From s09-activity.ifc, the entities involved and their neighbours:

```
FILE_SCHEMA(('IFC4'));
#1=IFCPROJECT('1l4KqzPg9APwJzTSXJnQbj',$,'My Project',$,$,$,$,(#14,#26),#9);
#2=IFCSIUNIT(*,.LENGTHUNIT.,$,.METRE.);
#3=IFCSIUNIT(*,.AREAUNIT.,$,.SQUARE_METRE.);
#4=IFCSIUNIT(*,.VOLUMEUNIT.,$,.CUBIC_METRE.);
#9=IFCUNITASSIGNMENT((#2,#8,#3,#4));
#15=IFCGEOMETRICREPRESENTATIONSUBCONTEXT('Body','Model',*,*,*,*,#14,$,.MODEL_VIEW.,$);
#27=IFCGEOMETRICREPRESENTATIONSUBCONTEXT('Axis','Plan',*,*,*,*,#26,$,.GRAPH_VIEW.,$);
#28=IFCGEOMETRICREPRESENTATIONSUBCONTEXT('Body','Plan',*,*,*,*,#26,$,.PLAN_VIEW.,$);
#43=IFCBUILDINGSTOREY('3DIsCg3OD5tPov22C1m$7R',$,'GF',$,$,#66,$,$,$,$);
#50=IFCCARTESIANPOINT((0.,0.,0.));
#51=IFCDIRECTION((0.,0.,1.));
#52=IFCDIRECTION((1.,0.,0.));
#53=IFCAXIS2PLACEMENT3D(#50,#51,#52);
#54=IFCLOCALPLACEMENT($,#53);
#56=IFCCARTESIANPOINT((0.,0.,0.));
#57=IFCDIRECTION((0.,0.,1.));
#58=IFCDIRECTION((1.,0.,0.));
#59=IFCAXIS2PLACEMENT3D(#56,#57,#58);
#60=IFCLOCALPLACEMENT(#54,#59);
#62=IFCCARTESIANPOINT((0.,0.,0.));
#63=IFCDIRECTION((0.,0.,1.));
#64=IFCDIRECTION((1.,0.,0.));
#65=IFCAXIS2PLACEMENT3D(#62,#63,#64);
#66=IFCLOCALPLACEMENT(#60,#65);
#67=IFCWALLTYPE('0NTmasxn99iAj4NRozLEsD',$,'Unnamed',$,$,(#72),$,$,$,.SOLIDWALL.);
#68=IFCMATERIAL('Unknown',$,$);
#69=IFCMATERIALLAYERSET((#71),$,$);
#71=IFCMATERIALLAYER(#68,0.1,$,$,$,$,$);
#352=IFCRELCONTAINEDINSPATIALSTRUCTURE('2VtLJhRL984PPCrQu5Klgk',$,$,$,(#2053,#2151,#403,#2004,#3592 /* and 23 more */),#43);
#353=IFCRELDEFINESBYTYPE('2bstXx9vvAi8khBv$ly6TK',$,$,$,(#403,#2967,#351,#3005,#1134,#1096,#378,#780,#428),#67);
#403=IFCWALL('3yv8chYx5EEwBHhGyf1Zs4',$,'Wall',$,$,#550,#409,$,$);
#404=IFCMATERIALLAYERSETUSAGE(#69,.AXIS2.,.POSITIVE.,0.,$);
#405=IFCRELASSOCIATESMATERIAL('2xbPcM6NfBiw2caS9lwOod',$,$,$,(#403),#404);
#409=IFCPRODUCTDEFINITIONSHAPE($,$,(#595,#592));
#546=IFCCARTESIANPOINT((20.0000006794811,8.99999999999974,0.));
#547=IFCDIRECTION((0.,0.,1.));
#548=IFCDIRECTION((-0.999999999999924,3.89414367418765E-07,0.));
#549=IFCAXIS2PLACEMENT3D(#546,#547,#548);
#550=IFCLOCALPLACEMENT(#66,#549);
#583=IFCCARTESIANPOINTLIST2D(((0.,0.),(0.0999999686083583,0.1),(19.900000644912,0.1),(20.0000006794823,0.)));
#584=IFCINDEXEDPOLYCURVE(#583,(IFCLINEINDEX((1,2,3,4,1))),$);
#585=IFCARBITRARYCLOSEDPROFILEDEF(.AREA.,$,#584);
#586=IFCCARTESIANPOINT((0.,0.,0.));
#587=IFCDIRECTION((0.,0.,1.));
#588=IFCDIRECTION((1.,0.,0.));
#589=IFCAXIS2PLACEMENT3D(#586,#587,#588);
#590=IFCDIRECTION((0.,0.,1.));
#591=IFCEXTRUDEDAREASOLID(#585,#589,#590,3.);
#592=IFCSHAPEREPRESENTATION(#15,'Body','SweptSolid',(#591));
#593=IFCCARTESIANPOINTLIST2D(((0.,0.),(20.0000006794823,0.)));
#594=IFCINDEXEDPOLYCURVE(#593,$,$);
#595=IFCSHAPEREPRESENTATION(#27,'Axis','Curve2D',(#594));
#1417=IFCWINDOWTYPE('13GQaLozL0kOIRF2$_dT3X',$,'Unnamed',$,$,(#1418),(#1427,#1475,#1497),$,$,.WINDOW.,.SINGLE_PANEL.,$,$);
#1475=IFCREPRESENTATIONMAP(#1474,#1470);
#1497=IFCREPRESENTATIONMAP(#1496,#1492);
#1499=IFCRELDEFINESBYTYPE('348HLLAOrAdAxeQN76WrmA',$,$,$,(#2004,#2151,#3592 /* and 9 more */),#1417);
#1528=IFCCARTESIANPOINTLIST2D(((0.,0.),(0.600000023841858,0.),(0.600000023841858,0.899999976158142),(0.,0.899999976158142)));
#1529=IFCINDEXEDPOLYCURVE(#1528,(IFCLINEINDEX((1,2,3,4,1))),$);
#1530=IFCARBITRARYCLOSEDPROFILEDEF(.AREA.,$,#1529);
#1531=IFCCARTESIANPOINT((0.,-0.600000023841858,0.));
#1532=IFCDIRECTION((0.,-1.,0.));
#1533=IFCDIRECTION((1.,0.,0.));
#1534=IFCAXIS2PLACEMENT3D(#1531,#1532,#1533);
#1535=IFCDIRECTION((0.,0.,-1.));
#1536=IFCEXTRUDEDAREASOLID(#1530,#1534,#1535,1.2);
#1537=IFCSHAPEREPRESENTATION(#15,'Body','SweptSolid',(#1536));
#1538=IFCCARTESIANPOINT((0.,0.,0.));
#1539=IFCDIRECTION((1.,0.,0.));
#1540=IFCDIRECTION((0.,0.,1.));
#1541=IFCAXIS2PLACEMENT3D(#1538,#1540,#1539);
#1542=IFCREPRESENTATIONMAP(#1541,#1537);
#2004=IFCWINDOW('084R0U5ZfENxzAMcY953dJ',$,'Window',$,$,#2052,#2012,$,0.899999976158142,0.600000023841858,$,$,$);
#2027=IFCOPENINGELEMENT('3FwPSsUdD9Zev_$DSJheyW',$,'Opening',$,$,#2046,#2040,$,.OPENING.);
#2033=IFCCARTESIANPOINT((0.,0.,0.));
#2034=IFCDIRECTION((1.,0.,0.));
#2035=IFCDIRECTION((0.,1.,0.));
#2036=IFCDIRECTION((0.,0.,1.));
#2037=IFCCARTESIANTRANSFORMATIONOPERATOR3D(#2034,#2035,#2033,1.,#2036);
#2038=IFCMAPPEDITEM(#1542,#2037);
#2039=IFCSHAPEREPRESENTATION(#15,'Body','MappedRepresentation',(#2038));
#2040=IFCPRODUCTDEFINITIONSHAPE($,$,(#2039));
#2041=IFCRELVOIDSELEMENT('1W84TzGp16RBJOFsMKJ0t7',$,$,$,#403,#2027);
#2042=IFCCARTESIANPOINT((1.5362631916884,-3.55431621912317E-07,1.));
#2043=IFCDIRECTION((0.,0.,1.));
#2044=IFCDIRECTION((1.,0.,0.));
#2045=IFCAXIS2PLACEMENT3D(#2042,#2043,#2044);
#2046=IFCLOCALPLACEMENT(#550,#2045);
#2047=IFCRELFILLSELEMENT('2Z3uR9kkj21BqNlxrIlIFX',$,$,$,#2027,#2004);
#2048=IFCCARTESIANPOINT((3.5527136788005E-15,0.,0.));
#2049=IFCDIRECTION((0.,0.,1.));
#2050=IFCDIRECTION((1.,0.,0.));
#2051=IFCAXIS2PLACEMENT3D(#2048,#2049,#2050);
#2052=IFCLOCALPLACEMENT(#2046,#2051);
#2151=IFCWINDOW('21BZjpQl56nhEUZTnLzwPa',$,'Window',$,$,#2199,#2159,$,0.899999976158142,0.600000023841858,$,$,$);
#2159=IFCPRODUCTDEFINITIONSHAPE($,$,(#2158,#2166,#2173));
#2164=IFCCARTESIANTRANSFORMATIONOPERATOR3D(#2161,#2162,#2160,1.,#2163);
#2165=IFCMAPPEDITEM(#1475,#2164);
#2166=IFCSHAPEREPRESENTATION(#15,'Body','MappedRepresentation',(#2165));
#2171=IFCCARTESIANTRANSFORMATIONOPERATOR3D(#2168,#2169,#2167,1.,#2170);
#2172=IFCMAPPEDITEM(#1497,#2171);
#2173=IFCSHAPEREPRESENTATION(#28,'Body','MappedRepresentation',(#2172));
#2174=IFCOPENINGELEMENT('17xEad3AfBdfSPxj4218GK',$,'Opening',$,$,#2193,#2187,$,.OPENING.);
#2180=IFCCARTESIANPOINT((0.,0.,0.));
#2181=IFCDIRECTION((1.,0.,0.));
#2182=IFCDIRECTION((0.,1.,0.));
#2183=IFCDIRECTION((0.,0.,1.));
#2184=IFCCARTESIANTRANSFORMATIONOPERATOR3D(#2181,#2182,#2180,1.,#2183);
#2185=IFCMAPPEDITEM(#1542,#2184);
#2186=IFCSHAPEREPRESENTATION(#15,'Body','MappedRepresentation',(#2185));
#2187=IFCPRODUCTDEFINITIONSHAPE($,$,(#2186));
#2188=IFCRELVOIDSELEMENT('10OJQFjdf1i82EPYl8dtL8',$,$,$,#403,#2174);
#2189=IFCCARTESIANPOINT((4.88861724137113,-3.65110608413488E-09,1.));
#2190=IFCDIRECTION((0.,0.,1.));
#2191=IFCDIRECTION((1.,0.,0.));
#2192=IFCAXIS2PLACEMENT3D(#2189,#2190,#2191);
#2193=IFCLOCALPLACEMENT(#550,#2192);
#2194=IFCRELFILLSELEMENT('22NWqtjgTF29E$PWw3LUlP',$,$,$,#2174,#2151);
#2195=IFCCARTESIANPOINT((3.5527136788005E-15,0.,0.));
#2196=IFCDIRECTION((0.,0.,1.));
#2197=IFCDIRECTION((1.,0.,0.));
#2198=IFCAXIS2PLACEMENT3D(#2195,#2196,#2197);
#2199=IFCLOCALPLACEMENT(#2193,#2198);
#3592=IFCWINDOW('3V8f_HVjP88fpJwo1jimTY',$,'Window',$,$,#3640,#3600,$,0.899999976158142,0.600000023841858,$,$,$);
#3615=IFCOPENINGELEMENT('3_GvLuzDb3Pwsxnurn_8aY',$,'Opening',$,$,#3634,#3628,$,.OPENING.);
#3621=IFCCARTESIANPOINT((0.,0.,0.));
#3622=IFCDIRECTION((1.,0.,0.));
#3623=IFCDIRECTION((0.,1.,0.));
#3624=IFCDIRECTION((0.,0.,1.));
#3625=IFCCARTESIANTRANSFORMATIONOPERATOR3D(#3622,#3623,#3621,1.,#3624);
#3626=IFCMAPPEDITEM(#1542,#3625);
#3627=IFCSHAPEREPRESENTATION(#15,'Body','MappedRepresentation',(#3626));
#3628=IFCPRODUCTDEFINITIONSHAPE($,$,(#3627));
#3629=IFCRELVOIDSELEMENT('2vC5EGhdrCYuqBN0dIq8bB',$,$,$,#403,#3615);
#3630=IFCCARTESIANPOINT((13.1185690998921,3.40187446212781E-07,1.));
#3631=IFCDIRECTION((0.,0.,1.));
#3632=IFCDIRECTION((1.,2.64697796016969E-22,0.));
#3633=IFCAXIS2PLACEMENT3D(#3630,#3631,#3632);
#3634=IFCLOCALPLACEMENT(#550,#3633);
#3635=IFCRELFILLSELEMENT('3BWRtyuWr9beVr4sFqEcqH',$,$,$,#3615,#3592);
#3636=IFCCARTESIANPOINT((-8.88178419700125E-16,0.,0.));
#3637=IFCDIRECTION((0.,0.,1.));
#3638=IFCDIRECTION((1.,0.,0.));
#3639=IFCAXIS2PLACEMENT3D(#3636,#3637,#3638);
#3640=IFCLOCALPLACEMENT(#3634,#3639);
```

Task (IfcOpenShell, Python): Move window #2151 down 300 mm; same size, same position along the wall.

```python
import numpy as np
import ifcopenshell
import ifcopenshell.api.geometry
import ifcopenshell.util.placement
import ifcopenshell.util.unit

model = ifcopenshell.open("s09-activity.ifc")
unit_scale = ifcopenshell.util.unit.calculate_unit_scale(model)

window = model.by_id(2151)
opening = window.FillsVoids[0].RelatingOpeningElement
dz = -0.3

shift = np.array([0.0, 0.0, dz])
# The window is placed relative to its opening, so it follows when the opening moves.
matrix = ifcopenshell.util.placement.get_local_placement(opening.ObjectPlacement)
matrix[:3, 3] += shift
ifcopenshell.api.geometry.edit_object_placement(
    model, product=opening, matrix=matrix, is_si=False, should_transform_children=True
)

print(f"moved by {dz * unit_scale:+.3f} m")

model.write("s09-activity_updated.ifc")
```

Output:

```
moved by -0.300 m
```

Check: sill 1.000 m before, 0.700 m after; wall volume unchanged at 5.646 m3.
